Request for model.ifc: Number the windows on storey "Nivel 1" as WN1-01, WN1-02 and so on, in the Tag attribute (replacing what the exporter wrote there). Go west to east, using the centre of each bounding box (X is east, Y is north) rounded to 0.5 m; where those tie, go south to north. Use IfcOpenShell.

First a look at what the model holds.

```python
import ifcopenshell
import ifcopenshell.util.element
import ifcopenshell.util.placement

model = ifcopenshell.open("model.ifc")
print(model.schema)
storey = next(s for s in model.by_type("IfcBuildingStorey") if s.Name == "Nivel 1")
windows = [e for e in ifcopenshell.util.element.get_decomposition(storey) if e.is_a("IfcWindow")]
for e in sorted(windows, key=lambda e: e.id()):
    origin = ifcopenshell.util.placement.get_local_placement(e.ObjectPlacement)[:3, 3]
    print(e.id(), e.Tag, e.Name, origin.round(2) + 0.0, sep=" | ")
```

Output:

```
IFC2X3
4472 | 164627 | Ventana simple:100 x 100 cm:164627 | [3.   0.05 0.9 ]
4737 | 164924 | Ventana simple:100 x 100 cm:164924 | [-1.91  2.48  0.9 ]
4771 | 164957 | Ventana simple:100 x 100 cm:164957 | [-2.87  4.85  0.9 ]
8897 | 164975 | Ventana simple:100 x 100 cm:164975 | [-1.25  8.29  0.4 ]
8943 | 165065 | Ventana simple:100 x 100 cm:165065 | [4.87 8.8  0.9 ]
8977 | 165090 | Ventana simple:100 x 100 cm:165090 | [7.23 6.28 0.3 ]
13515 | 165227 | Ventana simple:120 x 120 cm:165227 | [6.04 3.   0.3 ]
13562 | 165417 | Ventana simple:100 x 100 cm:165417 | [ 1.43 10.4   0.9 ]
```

```python
import ifcopenshell
import ifcopenshell.geom
import ifcopenshell.util.element
import ifcopenshell.util.shape

model = ifcopenshell.open("model.ifc")
settings = ifcopenshell.geom.settings()
settings.set("use-world-coords", True)


def centre(element):
    shape = ifcopenshell.geom.create_shape(settings, element)
    return ifcopenshell.util.shape.get_bbox_centroid(shape.geometry)


storey = next(s for s in model.by_type("IfcBuildingStorey") if s.Name == "Nivel 1")
windows = [e for e in ifcopenshell.util.element.get_decomposition(storey) if e.is_a("IfcWindow")]

# Insertion points can sit at a corner or the storey origin, so sort by the geometry (in metres).
centres = {e: centre(e) for e in windows}
windows.sort(key=lambda e: (round(centres[e][0] / 0.5), centres[e][1]))

for i, e in enumerate(windows, start=1):
    number = f"WN1-{i:02d}"
    e.Tag = number
    print(e.id(), number)

model.write("model-out.ifc")
```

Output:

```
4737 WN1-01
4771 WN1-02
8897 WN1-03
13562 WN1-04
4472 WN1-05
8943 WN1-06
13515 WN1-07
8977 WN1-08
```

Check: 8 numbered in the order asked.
